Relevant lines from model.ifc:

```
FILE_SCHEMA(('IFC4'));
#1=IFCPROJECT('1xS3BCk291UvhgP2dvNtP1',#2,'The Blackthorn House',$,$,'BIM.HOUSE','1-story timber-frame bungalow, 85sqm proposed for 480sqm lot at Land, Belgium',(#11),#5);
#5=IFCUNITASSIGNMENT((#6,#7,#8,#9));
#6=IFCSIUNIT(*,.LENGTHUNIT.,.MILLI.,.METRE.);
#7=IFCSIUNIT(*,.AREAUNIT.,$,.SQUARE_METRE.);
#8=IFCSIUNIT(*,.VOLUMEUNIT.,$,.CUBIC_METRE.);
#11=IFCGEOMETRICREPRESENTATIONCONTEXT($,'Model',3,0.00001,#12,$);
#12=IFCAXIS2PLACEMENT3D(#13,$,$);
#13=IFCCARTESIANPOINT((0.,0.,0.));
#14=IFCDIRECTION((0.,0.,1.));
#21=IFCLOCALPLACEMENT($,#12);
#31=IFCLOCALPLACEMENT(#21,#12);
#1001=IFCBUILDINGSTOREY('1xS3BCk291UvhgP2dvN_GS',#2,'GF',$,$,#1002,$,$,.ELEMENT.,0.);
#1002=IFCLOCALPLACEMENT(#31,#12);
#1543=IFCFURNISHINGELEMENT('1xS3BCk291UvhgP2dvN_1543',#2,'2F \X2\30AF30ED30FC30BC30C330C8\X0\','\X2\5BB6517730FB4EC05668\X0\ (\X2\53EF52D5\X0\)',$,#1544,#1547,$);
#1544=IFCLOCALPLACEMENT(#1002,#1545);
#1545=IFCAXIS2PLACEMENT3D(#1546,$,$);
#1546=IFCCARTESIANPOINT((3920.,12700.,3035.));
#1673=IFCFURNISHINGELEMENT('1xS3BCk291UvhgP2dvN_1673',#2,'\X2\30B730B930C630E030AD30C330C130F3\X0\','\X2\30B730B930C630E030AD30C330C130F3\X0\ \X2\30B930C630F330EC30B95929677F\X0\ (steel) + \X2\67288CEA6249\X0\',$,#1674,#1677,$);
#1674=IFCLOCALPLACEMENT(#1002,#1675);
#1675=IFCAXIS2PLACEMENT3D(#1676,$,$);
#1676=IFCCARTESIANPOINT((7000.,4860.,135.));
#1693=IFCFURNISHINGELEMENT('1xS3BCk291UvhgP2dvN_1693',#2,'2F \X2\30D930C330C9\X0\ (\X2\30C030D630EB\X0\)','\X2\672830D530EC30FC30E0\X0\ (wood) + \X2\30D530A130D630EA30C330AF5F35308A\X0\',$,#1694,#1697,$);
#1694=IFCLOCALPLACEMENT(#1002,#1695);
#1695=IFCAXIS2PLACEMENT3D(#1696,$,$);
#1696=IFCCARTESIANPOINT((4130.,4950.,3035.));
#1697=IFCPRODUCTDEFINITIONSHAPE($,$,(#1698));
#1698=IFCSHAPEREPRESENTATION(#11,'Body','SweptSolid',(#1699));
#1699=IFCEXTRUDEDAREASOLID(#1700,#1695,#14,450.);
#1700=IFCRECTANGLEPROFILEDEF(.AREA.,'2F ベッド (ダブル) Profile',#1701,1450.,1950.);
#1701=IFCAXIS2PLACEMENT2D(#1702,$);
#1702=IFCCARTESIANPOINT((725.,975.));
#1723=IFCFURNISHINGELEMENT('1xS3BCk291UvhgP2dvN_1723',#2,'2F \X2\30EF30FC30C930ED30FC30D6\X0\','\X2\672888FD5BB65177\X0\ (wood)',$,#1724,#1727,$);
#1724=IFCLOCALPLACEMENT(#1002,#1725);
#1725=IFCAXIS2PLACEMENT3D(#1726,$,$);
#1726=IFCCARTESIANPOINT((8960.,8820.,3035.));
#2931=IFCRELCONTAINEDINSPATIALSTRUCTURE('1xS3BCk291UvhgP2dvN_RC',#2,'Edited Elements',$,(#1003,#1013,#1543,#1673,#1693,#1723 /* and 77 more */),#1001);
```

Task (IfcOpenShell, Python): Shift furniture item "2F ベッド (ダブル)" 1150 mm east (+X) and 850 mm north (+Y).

```python
import ifcopenshell
import ifcopenshell.api.geometry
import ifcopenshell.util.placement
import ifcopenshell.util.unit

model = ifcopenshell.open("model.ifc")
unit_scale = ifcopenshell.util.unit.calculate_unit_scale(model)

item = model.by_id(1693)
matrix = ifcopenshell.util.placement.get_local_placement(item.ObjectPlacement)
matrix[0, 3] += 1.15 / unit_scale
matrix[1, 3] += 0.85 / unit_scale
ifcopenshell.api.geometry.edit_object_placement(model, product=item, matrix=matrix, is_si=False)

print(ifcopenshell.util.placement.get_local_placement(item.ObjectPlacement).round(3) + 0.0)

model.write("model_edited.ifc")
```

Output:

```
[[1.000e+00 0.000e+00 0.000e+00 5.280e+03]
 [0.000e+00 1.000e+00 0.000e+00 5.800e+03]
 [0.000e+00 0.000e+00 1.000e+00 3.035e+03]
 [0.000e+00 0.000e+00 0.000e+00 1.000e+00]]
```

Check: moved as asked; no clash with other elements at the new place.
